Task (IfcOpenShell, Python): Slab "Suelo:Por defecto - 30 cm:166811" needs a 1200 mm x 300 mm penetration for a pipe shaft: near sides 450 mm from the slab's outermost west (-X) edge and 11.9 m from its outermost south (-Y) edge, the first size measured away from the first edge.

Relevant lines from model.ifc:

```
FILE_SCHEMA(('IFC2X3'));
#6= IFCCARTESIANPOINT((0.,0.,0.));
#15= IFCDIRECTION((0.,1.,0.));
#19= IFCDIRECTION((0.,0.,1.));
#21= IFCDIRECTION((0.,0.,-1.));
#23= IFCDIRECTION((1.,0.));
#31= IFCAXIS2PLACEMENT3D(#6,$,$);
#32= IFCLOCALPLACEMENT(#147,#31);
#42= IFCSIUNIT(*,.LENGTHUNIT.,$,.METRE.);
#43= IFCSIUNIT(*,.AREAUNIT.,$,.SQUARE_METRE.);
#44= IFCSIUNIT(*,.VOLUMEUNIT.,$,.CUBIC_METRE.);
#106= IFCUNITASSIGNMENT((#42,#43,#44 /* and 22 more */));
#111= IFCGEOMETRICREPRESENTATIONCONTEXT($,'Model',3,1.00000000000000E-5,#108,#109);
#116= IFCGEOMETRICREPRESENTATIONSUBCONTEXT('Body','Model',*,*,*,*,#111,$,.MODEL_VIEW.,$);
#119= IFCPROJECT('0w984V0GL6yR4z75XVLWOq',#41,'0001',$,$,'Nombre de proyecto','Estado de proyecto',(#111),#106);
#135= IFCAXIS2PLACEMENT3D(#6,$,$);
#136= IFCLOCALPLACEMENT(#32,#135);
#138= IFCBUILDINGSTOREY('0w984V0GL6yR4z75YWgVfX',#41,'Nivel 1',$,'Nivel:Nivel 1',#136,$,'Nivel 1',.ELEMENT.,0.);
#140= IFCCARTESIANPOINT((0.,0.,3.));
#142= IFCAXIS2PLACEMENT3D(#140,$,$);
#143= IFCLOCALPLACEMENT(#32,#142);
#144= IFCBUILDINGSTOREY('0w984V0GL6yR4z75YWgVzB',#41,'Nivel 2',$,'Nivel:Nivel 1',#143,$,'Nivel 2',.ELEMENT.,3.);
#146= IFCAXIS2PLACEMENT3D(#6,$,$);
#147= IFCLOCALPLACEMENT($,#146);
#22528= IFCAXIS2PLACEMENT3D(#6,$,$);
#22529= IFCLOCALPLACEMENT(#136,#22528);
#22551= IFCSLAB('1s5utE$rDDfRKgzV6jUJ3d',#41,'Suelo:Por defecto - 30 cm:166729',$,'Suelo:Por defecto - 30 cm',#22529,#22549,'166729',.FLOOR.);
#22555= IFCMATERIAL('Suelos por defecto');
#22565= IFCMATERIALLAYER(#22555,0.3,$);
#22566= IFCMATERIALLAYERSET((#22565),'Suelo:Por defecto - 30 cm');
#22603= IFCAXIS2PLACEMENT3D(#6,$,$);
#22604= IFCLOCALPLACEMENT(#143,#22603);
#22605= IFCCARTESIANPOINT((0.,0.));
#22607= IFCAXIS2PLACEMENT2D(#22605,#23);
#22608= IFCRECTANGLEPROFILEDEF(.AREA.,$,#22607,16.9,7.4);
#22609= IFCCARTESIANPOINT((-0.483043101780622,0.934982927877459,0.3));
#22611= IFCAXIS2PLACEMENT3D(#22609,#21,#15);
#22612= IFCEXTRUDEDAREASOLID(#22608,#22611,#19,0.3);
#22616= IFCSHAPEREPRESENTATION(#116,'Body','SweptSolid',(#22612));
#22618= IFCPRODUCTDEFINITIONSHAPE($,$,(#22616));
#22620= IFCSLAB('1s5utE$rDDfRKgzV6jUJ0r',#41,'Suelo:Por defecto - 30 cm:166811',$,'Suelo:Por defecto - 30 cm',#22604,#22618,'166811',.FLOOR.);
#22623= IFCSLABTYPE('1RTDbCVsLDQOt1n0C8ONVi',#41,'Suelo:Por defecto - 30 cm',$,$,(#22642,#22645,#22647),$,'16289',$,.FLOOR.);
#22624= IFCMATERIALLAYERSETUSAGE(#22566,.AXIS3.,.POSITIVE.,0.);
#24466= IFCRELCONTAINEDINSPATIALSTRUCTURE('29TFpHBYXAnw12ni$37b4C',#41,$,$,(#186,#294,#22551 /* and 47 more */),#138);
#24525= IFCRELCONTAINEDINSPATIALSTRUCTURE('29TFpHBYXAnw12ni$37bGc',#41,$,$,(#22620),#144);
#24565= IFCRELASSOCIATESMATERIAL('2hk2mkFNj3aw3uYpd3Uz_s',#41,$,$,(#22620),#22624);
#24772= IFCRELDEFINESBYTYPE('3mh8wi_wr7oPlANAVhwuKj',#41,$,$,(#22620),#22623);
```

```python
import numpy as np
import ifcopenshell
import ifcopenshell.api.feature
import ifcopenshell.api.geometry
import ifcopenshell.api.root
import ifcopenshell.geom
import ifcopenshell.util.placement
import ifcopenshell.util.representation
import ifcopenshell.util.shape
import ifcopenshell.util.unit

model = ifcopenshell.open("model.ifc")
unit_scale = ifcopenshell.util.unit.calculate_unit_scale(model)
settings = ifcopenshell.geom.settings()


def volume(element):
    """Net volume in cubic metres, openings subtracted."""
    shape = ifcopenshell.geom.create_shape(settings, element)
    return ifcopenshell.util.shape.get_volume(shape.geometry)


slab = model.by_guid("1s5utE$rDDfRKgzV6jUJ0r")
before = volume(slab)

# Extent in the slab's own axes, in metres. The edges named are its -X and -Y sides.
slab_shape = ifcopenshell.geom.create_shape(settings, slab)
vertices = ifcopenshell.util.shape.get_vertices(slab_shape.geometry)
x_min, y_min, bottom = vertices.min(axis=0)
top = vertices[:, 2].max()

opening = ifcopenshell.api.root.create_entity(model, ifc_class="IfcOpeningElement", name="Pipe shaft opening")
context = ifcopenshell.util.representation.get_context(model, "Model", "Body", "MODEL_VIEW")
width, depth = 1.2, 0.3
outline = [(0.0, 0.0), (width, 0.0), (width, depth), (0.0, depth), (0.0, 0.0)]
# Overshoot both faces by 50 mm so the cut is clean.
shape = ifcopenshell.api.geometry.add_slab_representation(
    model, context=context, depth=top - bottom + 0.1, polyline=outline
)
ifcopenshell.api.geometry.assign_representation(model, product=opening, representation=shape)

matrix = ifcopenshell.util.placement.get_local_placement(slab.ObjectPlacement)
matrix[:, 3] = matrix @ np.append(np.array([x_min + 0.45, y_min + 11.9, bottom - 0.05]) / unit_scale, 1.0)
ifcopenshell.api.geometry.edit_object_placement(model, product=opening, matrix=matrix, is_si=False)
ifcopenshell.api.feature.add_feature(model, feature=opening, element=slab)

after = volume(slab)

print(f"slab volume {before:.3f} -> {after:.3f} m3")

model.write("model_v2.ifc")
```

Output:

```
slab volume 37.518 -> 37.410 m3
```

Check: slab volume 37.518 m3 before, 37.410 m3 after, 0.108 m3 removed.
